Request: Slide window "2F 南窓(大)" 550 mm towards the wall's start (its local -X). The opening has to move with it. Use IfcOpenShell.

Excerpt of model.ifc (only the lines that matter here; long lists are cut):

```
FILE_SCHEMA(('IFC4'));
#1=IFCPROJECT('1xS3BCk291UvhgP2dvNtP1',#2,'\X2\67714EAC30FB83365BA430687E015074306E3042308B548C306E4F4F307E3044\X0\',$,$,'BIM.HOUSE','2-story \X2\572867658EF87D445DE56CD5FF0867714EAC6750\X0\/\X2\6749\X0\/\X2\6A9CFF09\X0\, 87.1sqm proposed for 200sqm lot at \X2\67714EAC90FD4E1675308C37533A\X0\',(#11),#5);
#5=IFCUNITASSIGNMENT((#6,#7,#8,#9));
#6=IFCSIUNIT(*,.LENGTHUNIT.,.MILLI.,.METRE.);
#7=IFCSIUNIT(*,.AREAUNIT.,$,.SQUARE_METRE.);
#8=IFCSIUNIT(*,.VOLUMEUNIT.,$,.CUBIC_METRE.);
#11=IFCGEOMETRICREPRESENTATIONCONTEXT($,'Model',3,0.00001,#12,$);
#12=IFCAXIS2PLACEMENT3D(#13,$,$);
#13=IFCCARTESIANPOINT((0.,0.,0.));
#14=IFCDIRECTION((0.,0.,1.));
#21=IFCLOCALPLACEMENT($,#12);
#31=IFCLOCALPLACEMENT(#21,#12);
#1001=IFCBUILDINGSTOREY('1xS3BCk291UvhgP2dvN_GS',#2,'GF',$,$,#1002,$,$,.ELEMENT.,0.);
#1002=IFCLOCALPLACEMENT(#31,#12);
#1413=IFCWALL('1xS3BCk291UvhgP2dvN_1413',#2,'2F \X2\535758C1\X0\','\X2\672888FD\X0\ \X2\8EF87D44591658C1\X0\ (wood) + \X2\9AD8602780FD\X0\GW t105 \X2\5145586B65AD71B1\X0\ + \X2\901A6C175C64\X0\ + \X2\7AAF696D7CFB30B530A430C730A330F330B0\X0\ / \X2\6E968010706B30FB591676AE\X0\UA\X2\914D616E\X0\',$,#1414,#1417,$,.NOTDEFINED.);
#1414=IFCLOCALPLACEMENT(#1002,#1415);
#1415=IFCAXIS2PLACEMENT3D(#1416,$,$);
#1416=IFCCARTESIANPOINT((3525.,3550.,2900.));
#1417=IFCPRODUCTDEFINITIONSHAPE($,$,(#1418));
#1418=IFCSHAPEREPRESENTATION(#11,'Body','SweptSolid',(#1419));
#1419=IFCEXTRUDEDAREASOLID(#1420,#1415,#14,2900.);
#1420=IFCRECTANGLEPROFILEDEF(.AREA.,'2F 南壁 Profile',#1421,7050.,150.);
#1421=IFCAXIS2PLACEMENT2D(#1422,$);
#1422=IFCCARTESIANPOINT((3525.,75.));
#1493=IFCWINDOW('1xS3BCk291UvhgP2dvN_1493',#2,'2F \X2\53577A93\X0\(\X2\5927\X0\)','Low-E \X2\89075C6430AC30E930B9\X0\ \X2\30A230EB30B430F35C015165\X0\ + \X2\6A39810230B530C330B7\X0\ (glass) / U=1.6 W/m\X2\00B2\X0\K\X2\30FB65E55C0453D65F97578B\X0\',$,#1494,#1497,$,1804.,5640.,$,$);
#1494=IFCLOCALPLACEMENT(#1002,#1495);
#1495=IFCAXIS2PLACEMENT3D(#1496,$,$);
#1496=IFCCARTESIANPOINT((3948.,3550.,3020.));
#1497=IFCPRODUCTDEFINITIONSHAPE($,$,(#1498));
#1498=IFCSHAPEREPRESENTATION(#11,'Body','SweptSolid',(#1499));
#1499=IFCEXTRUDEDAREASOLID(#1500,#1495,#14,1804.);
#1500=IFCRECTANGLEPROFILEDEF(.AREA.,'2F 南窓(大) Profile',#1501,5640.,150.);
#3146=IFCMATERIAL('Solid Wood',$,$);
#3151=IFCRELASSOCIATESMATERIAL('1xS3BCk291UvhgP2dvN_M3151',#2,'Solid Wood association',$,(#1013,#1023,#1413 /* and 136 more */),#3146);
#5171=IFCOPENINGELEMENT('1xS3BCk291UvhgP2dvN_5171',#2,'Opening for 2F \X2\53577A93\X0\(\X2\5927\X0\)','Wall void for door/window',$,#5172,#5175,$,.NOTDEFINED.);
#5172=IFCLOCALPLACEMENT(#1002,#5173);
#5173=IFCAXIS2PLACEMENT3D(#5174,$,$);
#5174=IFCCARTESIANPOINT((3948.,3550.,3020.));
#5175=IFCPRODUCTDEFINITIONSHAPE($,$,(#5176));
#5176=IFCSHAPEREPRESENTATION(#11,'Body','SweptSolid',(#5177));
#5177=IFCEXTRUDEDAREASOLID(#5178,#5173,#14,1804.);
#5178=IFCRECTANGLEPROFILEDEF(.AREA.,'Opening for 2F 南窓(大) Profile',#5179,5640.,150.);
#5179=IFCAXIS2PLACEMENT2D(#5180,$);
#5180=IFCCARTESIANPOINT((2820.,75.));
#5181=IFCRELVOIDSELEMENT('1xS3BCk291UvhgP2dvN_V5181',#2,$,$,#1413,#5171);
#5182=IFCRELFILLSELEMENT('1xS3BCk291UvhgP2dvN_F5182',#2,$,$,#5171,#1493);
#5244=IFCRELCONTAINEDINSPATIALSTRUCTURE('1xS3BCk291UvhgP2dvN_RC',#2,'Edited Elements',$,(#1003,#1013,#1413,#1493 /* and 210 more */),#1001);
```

```python
import ifcopenshell
import ifcopenshell.api.geometry
import ifcopenshell.util.placement
import ifcopenshell.util.unit

model = ifcopenshell.open("model.ifc")
unit_scale = ifcopenshell.util.unit.calculate_unit_scale(model)

window = model.by_guid("1xS3BCk291UvhgP2dvN_1493")
opening = window.FillsVoids[0].RelatingOpeningElement
wall = opening.VoidsElements[0].RelatingBuildingElement

wall_matrix = ifcopenshell.util.placement.get_local_placement(wall.ObjectPlacement)
shift = wall_matrix[:3, 0] * -0.55 / unit_scale
before = ifcopenshell.util.placement.get_local_placement(window.ObjectPlacement)[:3, 3].copy()

# The window is not placed relative to its opening, so move both.
for product in (opening, window):
    matrix = ifcopenshell.util.placement.get_local_placement(product.ObjectPlacement)
    matrix[:3, 3] += shift
    ifcopenshell.api.geometry.edit_object_placement(model, product=product, matrix=matrix, is_si=False)

after = ifcopenshell.util.placement.get_local_placement(window.ObjectPlacement)[:3, 3]
print("window moved by", (after - before).round(3) + 0.0)

model.write("model_v2.ifc")
```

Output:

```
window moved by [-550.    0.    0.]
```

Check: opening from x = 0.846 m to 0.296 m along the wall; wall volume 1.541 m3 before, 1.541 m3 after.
